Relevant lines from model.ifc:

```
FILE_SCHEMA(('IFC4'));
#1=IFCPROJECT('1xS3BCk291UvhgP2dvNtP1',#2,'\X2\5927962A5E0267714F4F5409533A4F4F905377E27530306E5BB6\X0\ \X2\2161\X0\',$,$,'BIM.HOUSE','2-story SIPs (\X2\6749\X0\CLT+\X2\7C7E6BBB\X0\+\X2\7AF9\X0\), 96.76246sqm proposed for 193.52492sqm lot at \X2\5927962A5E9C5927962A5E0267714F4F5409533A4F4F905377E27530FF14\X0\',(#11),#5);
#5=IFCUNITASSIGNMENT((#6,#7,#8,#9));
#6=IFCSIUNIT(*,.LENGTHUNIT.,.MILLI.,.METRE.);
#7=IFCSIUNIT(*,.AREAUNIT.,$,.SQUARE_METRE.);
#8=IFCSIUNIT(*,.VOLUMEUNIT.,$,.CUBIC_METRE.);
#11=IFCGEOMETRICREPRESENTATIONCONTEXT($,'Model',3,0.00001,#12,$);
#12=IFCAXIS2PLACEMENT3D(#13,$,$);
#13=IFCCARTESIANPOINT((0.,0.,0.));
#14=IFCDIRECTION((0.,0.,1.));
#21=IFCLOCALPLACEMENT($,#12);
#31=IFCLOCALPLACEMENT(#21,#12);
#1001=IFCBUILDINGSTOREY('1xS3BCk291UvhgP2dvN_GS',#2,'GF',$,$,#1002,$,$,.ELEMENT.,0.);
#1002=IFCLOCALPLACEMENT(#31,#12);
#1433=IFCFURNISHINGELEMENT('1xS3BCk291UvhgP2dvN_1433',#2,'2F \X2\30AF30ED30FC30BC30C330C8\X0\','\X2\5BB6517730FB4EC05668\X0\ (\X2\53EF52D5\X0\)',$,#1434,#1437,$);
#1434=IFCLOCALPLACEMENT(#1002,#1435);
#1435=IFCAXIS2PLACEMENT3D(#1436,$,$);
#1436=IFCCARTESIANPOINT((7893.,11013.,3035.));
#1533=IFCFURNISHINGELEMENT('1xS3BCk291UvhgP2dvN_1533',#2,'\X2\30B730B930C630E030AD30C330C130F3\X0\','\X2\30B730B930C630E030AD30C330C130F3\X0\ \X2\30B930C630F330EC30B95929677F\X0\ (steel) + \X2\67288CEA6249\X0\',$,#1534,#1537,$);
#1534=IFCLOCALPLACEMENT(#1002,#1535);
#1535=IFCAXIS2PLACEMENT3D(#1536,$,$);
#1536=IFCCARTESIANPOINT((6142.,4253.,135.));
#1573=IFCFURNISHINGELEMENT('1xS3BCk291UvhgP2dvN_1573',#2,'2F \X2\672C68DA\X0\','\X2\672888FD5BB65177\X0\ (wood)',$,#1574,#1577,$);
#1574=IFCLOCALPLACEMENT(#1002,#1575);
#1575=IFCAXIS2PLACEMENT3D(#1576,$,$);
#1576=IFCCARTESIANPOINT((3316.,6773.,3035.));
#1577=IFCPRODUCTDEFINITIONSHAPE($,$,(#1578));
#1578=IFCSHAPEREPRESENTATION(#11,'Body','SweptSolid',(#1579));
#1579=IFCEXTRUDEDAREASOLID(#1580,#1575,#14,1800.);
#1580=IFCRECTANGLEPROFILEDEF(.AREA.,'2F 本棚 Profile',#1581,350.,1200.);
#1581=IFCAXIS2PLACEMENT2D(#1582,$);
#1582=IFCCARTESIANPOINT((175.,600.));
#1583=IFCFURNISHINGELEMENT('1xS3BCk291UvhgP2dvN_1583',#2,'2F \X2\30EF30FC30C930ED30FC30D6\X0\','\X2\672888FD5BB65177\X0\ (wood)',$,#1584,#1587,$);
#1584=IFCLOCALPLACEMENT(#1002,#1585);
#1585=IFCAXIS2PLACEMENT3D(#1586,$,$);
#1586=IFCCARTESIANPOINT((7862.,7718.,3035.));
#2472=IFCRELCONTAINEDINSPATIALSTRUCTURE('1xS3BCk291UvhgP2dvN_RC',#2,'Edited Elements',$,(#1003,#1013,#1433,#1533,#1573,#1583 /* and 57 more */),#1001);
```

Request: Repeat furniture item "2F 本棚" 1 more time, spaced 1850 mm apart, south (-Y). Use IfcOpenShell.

```python
import numpy as np
import ifcopenshell
import ifcopenshell.api.geometry
import ifcopenshell.api.root
import ifcopenshell.util.element
import ifcopenshell.util.placement
import ifcopenshell.util.unit

model = ifcopenshell.open("model.ifc")
unit_scale = ifcopenshell.util.unit.calculate_unit_scale(model)


def reuse_history(source, copy):
    """copy_class also copies each property set's owner history, people and application; keep the originals."""
    for rel in copy.IsDefinedBy:
        if rel.is_a("IfcRelDefinesByProperties") and (history := rel.RelatingPropertyDefinition.OwnerHistory):
            rel.RelatingPropertyDefinition.OwnerHistory = source.OwnerHistory
            ifcopenshell.util.element.remove_deep2(model, history)


source = model.by_guid("1xS3BCk291UvhgP2dvN_1573")
base = ifcopenshell.util.placement.get_local_placement(source.ObjectPlacement)
step = np.array([0.0, -1.0, 0.0]) * 1.85 / unit_scale

for i in range(1, 2):
    copy = ifcopenshell.api.root.copy_class(model, product=source)
    copy.Representation = ifcopenshell.util.element.copy_deep(
        model, source.Representation, exclude=["IfcGeometricRepresentationContext", "IfcRepresentationMap"]
    )
    reuse_history(source, copy)
    matrix = base.copy()
    matrix[:3, 3] += i * step
    print("added at", matrix[:3, 3].round(3) + 0.0)
    ifcopenshell.api.geometry.edit_object_placement(model, product=copy, matrix=matrix, is_si=False)

model.write("model_updated.ifc")
```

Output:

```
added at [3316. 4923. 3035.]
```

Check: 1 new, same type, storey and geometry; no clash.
